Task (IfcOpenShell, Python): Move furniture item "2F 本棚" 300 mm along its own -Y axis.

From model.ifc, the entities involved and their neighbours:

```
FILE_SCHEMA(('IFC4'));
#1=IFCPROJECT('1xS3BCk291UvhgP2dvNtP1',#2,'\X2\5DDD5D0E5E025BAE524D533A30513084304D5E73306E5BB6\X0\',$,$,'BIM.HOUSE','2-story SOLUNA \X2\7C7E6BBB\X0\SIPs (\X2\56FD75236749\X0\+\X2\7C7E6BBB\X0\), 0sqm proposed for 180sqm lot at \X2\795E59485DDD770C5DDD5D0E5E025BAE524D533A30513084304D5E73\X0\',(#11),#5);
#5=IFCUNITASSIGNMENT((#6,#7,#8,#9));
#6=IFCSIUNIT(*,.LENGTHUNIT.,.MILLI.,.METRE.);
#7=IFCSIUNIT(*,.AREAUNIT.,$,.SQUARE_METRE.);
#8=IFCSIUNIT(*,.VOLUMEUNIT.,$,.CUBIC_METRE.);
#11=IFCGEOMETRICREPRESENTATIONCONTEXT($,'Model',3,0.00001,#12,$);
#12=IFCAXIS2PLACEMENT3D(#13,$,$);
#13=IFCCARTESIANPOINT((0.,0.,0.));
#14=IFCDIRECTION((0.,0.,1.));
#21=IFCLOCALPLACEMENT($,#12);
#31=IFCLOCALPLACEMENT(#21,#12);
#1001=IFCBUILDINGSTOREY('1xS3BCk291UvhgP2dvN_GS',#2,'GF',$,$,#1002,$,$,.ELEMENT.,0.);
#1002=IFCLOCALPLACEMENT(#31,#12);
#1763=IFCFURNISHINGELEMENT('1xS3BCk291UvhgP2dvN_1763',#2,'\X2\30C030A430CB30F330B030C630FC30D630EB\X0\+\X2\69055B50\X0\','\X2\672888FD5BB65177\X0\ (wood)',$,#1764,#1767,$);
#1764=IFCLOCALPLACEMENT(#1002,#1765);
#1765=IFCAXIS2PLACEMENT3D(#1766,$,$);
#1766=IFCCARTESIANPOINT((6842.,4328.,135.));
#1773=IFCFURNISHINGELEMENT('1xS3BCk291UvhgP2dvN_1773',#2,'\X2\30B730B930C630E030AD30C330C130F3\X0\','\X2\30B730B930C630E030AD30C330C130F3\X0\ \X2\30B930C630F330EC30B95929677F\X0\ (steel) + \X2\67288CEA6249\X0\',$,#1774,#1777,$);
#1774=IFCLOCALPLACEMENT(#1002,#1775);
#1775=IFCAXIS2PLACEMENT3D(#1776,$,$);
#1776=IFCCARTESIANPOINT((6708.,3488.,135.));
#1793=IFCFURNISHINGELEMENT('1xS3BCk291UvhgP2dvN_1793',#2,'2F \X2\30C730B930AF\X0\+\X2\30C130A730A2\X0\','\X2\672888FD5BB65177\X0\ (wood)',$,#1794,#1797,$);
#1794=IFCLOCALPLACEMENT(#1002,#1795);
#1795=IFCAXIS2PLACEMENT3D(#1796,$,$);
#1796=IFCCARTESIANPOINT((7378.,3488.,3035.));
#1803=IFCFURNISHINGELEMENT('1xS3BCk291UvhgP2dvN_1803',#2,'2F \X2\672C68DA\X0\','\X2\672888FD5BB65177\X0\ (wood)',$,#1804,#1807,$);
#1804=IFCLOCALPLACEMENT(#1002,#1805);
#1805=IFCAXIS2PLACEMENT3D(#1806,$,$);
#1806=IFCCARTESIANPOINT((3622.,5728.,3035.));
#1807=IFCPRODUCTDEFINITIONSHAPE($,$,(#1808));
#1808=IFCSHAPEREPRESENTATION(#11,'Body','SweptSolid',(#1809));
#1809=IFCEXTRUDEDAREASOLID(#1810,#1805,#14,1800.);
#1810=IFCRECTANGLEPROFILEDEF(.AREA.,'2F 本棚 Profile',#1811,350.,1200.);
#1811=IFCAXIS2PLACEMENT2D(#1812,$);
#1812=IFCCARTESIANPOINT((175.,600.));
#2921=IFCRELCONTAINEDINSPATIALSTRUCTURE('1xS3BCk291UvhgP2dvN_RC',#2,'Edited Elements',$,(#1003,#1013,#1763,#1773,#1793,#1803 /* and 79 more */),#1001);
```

```python
import ifcopenshell
import ifcopenshell.api.geometry
import ifcopenshell.util.placement
import ifcopenshell.util.unit

model = ifcopenshell.open("model.ifc")
unit_scale = ifcopenshell.util.unit.calculate_unit_scale(model)

item = model.by_guid("1xS3BCk291UvhgP2dvN_1803")
matrix = ifcopenshell.util.placement.get_local_placement(item.ObjectPlacement)
matrix[:3, 3] -= matrix[:3, 1] * 0.3 / unit_scale
ifcopenshell.api.geometry.edit_object_placement(model, product=item, matrix=matrix, is_si=False)

print(ifcopenshell.util.placement.get_local_placement(item.ObjectPlacement).round(3) + 0.0)

model.write("model_v2.ifc")
```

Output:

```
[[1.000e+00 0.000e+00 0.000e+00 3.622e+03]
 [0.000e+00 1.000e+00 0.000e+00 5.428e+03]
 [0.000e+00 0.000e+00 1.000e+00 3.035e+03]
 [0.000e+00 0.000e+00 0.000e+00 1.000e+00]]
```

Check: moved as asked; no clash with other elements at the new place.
